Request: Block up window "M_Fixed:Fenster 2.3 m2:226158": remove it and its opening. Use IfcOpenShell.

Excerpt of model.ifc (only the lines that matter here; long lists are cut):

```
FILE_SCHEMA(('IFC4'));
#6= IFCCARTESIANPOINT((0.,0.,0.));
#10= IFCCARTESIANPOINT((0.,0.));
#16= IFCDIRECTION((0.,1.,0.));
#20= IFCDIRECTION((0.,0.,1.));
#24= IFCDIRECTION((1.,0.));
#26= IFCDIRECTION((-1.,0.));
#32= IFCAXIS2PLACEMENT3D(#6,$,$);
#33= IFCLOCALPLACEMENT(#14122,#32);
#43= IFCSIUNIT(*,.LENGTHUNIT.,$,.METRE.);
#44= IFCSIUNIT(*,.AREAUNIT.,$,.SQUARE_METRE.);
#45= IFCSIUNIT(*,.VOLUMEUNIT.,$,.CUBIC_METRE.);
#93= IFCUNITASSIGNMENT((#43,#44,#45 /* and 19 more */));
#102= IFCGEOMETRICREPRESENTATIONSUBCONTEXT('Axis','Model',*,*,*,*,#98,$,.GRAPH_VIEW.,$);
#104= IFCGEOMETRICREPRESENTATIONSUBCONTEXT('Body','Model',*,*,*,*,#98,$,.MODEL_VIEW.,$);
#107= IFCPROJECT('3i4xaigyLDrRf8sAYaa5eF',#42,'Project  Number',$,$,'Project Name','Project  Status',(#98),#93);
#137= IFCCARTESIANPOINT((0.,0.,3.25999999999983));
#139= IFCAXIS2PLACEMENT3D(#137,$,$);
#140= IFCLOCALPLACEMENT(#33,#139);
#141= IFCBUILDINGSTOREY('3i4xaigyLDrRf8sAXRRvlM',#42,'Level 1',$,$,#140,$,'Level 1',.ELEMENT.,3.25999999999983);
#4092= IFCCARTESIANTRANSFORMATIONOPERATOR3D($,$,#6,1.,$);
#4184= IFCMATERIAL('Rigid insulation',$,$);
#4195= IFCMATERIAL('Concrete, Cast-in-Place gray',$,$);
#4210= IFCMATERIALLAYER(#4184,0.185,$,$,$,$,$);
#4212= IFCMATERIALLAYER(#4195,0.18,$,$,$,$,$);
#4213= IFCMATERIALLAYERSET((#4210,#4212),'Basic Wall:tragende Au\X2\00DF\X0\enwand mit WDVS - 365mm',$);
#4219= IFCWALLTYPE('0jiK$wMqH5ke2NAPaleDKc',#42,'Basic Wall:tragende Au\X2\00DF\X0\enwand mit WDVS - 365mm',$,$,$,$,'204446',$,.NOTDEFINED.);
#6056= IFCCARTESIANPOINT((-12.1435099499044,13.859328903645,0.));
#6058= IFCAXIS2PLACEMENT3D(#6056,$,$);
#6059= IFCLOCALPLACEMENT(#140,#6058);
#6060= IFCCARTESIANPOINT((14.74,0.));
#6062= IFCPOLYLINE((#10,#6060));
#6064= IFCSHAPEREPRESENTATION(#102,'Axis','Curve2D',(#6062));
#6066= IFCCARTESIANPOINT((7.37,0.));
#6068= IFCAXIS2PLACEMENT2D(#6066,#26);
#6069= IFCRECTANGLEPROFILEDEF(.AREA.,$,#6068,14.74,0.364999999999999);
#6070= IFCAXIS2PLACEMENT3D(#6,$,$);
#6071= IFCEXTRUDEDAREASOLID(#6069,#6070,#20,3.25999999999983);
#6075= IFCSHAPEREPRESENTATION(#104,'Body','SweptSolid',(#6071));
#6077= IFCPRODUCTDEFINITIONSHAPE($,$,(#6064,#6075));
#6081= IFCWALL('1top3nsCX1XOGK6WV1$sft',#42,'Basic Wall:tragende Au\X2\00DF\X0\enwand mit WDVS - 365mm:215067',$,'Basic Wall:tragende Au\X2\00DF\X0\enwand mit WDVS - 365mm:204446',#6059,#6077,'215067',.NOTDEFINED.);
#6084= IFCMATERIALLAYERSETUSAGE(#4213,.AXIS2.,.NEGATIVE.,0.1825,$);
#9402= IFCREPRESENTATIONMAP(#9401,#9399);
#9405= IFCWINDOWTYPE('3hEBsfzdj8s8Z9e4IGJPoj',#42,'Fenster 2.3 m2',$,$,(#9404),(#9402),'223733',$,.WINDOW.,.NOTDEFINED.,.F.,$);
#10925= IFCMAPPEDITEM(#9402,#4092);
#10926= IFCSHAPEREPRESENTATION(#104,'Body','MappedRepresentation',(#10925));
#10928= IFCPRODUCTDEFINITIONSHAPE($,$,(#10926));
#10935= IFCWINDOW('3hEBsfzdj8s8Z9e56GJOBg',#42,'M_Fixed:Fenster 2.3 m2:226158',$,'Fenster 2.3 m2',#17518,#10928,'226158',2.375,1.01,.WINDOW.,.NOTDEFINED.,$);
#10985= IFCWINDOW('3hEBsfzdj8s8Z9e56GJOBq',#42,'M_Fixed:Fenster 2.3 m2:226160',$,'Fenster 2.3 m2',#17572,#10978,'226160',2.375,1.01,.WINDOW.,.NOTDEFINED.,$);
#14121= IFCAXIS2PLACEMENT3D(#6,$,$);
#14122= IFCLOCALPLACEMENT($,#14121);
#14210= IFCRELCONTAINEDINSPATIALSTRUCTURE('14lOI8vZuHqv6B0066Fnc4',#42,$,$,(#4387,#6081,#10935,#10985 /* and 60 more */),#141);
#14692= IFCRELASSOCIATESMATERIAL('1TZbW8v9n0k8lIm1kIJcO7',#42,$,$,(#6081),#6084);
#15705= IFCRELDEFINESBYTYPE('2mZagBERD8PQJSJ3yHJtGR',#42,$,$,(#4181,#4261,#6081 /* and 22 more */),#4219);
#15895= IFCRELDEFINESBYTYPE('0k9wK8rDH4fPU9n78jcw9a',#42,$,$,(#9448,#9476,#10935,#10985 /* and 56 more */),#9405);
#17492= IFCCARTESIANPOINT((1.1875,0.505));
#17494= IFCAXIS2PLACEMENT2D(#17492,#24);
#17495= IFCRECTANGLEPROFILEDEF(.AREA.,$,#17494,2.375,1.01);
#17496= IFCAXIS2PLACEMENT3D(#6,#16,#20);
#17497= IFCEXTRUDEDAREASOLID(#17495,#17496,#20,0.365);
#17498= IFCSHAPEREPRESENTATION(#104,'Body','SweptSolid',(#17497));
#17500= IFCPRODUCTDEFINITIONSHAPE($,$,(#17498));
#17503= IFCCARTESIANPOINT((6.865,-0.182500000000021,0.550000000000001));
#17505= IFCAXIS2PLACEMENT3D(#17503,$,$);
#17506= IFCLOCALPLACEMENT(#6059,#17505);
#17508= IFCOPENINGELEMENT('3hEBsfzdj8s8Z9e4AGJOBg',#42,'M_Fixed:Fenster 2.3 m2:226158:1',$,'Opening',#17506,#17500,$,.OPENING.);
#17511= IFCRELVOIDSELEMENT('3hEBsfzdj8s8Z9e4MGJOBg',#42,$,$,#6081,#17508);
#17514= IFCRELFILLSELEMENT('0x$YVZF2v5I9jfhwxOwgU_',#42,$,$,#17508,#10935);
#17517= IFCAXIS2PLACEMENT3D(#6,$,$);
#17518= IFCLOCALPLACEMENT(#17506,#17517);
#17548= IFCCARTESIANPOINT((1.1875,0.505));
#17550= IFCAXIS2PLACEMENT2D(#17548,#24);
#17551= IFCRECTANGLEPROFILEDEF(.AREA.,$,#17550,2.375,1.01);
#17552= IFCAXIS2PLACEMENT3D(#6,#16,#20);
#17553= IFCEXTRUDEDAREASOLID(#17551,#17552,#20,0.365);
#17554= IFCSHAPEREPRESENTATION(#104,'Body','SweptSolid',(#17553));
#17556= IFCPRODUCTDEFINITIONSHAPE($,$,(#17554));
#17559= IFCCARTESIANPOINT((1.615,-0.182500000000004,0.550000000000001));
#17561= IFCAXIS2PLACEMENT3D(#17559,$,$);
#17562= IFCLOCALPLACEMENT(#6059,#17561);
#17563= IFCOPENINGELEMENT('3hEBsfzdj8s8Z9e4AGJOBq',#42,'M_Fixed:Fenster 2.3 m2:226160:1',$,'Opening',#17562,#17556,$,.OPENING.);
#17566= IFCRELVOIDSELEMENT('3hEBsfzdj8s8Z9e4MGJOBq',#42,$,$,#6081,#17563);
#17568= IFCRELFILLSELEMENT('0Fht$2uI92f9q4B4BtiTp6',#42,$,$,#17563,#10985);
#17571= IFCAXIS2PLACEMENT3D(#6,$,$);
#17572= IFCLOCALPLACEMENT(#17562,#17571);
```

```python
import ifcopenshell
import ifcopenshell.api.feature
import ifcopenshell.api.root
import ifcopenshell.geom
import ifcopenshell.util.shape

model = ifcopenshell.open("model.ifc")
settings = ifcopenshell.geom.settings()


def volume(element):
    """Net volume in cubic metres, openings subtracted."""
    shape = ifcopenshell.geom.create_shape(settings, element)
    return ifcopenshell.util.shape.get_volume(shape.geometry)


window = model.by_guid("3hEBsfzdj8s8Z9e56GJOBg")
opening = window.FillsVoids[0].RelatingOpeningElement
wall = opening.VoidsElements[0].RelatingBuildingElement
before = volume(wall)

ifcopenshell.api.root.remove_product(model, product=window)
ifcopenshell.api.feature.remove_feature(model, feature=opening)

after = volume(wall)

print(f"wall volume {before:.3f} -> {after:.3f} m3")

model.write("model_v2.ifc")
```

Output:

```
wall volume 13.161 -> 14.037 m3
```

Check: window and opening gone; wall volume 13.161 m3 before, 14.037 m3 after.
